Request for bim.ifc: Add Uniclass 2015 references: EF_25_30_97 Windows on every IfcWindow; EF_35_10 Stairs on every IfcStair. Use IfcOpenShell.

First a look at what the model holds.

```python
import ifcopenshell

model = ifcopenshell.open("bim.ifc")
print(model.schema)
print("classifications:", [c.Name for c in model.by_type("IfcClassification")])
for ifc_class in ("IfcDoor", "IfcRoof", "IfcStair", "IfcWall", "IfcWindow"):
    print(ifc_class, len(model.by_type(ifc_class)))
```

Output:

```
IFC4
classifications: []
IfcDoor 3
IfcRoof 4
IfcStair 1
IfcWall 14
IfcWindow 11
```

```python
import ifcopenshell
import ifcopenshell.api.classification

model = ifcopenshell.open("bim.ifc")

system = ifcopenshell.api.classification.add_classification(model, classification="Uniclass 2015")

codes = {
    "IfcWindow": ("EF_25_30_97", "Windows"),
    "IfcStair": ("EF_35_10", "Stairs"),
}
for ifc_class, (code, name) in codes.items():
    products = model.by_type(ifc_class)
    ifcopenshell.api.classification.add_reference(
        model, products=products, classification=system, identification=code, name=name
    )
    print(code, len(products))

model.write("bim_rev.ifc")
```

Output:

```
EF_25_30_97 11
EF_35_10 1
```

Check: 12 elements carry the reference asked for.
